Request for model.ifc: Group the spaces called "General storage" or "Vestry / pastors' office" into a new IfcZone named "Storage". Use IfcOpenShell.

First a look at what the model holds.

```python
import ifcopenshell

model = ifcopenshell.open("model.ifc")
print(model.schema)
seen = {}
for space in model.by_type("IfcSpace"):
    seen[space.LongName] = seen.get(space.LongName, 0) + 1
for name, count in sorted(seen.items(), key=str):
    print(count, "x", name)
print("zones:", [z.Name for z in model.by_type("IfcZone")][:20])
```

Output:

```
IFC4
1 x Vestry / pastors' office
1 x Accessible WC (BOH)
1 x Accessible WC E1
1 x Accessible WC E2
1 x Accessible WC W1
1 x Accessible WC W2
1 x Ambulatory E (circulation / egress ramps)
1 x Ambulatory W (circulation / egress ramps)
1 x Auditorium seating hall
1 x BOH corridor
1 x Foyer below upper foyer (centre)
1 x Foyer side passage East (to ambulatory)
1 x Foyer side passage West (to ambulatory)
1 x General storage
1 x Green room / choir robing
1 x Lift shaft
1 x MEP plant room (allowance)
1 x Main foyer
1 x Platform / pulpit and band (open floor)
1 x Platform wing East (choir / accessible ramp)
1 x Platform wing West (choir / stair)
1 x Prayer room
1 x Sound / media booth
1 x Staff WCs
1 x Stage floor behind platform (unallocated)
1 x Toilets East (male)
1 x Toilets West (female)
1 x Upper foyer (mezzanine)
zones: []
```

```python
import ifcopenshell
import ifcopenshell.api.group
import ifcopenshell.api.root

model = ifcopenshell.open("model.ifc")

names = {"General storage", "Vestry / pastors' office"}
spaces = [s for s in model.by_type("IfcSpace") if s.LongName in names]

zone = ifcopenshell.api.root.create_entity(model, ifc_class="IfcZone", name="Storage")
ifcopenshell.api.group.assign_group(model, products=spaces, group=zone)
print(len(spaces), "spaces in", zone.Name)

model.write("model_v2.ifc")
```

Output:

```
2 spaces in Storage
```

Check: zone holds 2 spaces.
